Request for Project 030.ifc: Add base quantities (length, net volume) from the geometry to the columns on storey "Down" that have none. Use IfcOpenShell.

First a look at what the model holds.

```python
import ifcopenshell
import ifcopenshell.util.element
import ifcopenshell.util.unit

model = ifcopenshell.open("Project 030.ifc")
print(model.schema)
for unit_type in ("LENGTHUNIT", "AREAUNIT", "VOLUMEUNIT"):
    print(unit_type, ifcopenshell.util.unit.calculate_unit_scale(model, unit_type))
storey = next(s for s in model.by_type("IfcBuildingStorey") if s.Name == "Down")
columns = [e for e in ifcopenshell.util.element.get_decomposition(storey) if e.is_a("IfcColumn")]
for e in sorted(columns, key=lambda e: e.id()):
    print(e.id(), e.is_a(), e.Name, list(ifcopenshell.util.element.get_psets(e, qtos_only=True)), sep=" | ")
```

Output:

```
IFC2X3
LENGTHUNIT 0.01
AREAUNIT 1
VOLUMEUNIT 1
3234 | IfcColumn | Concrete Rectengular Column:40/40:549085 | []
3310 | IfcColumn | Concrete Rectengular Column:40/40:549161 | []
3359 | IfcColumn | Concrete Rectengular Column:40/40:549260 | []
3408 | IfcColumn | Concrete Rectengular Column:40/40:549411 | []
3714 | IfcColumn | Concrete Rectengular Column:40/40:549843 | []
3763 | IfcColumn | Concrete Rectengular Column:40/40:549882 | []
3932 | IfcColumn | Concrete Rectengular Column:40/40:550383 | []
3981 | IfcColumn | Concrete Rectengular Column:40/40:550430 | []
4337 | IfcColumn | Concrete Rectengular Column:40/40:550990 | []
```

```python
import ifcopenshell
import ifcopenshell.api.pset
import ifcopenshell.geom
import ifcopenshell.util.element
import ifcopenshell.util.shape
import ifcopenshell.util.unit

model = ifcopenshell.open("Project 030.ifc")
unit_scale = ifcopenshell.util.unit.calculate_unit_scale(model)
volume_scale = ifcopenshell.util.unit.calculate_unit_scale(model, "VOLUMEUNIT")
settings = ifcopenshell.geom.settings()

storey = next(s for s in model.by_type("IfcBuildingStorey") if s.Name == "Down")
columns = [e for e in ifcopenshell.util.element.get_decomposition(storey) if e.is_a("IfcColumn")]

for e in sorted(columns, key=lambda e: e.id()):
    if ifcopenshell.util.element.get_psets(e, qtos_only=True, should_inherit=False):
        continue
    # Geometry comes back in metres, in the element's own axes.
    shape = ifcopenshell.geom.create_shape(settings, e)
    values = {
        "Length": ifcopenshell.util.shape.get_z(shape.geometry) / unit_scale,
        "NetVolume": ifcopenshell.util.shape.get_volume(shape.geometry) / volume_scale,
    }
    qto = ifcopenshell.api.pset.add_qto(model, product=e, name="BaseQuantities")
    ifcopenshell.api.pset.edit_qto(model, qto=qto, properties=values)
    print(e.id(), {k: round(v, 3) for k, v in values.items()})

model.write("Project 030_v2.ifc")
```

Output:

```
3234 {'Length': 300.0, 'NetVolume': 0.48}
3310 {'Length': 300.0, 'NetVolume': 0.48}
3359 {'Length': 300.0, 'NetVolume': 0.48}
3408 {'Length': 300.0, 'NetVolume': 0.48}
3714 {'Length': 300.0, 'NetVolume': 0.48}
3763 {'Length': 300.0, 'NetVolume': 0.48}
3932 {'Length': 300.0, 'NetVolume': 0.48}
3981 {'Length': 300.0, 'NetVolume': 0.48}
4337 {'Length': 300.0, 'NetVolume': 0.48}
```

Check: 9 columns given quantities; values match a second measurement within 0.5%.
